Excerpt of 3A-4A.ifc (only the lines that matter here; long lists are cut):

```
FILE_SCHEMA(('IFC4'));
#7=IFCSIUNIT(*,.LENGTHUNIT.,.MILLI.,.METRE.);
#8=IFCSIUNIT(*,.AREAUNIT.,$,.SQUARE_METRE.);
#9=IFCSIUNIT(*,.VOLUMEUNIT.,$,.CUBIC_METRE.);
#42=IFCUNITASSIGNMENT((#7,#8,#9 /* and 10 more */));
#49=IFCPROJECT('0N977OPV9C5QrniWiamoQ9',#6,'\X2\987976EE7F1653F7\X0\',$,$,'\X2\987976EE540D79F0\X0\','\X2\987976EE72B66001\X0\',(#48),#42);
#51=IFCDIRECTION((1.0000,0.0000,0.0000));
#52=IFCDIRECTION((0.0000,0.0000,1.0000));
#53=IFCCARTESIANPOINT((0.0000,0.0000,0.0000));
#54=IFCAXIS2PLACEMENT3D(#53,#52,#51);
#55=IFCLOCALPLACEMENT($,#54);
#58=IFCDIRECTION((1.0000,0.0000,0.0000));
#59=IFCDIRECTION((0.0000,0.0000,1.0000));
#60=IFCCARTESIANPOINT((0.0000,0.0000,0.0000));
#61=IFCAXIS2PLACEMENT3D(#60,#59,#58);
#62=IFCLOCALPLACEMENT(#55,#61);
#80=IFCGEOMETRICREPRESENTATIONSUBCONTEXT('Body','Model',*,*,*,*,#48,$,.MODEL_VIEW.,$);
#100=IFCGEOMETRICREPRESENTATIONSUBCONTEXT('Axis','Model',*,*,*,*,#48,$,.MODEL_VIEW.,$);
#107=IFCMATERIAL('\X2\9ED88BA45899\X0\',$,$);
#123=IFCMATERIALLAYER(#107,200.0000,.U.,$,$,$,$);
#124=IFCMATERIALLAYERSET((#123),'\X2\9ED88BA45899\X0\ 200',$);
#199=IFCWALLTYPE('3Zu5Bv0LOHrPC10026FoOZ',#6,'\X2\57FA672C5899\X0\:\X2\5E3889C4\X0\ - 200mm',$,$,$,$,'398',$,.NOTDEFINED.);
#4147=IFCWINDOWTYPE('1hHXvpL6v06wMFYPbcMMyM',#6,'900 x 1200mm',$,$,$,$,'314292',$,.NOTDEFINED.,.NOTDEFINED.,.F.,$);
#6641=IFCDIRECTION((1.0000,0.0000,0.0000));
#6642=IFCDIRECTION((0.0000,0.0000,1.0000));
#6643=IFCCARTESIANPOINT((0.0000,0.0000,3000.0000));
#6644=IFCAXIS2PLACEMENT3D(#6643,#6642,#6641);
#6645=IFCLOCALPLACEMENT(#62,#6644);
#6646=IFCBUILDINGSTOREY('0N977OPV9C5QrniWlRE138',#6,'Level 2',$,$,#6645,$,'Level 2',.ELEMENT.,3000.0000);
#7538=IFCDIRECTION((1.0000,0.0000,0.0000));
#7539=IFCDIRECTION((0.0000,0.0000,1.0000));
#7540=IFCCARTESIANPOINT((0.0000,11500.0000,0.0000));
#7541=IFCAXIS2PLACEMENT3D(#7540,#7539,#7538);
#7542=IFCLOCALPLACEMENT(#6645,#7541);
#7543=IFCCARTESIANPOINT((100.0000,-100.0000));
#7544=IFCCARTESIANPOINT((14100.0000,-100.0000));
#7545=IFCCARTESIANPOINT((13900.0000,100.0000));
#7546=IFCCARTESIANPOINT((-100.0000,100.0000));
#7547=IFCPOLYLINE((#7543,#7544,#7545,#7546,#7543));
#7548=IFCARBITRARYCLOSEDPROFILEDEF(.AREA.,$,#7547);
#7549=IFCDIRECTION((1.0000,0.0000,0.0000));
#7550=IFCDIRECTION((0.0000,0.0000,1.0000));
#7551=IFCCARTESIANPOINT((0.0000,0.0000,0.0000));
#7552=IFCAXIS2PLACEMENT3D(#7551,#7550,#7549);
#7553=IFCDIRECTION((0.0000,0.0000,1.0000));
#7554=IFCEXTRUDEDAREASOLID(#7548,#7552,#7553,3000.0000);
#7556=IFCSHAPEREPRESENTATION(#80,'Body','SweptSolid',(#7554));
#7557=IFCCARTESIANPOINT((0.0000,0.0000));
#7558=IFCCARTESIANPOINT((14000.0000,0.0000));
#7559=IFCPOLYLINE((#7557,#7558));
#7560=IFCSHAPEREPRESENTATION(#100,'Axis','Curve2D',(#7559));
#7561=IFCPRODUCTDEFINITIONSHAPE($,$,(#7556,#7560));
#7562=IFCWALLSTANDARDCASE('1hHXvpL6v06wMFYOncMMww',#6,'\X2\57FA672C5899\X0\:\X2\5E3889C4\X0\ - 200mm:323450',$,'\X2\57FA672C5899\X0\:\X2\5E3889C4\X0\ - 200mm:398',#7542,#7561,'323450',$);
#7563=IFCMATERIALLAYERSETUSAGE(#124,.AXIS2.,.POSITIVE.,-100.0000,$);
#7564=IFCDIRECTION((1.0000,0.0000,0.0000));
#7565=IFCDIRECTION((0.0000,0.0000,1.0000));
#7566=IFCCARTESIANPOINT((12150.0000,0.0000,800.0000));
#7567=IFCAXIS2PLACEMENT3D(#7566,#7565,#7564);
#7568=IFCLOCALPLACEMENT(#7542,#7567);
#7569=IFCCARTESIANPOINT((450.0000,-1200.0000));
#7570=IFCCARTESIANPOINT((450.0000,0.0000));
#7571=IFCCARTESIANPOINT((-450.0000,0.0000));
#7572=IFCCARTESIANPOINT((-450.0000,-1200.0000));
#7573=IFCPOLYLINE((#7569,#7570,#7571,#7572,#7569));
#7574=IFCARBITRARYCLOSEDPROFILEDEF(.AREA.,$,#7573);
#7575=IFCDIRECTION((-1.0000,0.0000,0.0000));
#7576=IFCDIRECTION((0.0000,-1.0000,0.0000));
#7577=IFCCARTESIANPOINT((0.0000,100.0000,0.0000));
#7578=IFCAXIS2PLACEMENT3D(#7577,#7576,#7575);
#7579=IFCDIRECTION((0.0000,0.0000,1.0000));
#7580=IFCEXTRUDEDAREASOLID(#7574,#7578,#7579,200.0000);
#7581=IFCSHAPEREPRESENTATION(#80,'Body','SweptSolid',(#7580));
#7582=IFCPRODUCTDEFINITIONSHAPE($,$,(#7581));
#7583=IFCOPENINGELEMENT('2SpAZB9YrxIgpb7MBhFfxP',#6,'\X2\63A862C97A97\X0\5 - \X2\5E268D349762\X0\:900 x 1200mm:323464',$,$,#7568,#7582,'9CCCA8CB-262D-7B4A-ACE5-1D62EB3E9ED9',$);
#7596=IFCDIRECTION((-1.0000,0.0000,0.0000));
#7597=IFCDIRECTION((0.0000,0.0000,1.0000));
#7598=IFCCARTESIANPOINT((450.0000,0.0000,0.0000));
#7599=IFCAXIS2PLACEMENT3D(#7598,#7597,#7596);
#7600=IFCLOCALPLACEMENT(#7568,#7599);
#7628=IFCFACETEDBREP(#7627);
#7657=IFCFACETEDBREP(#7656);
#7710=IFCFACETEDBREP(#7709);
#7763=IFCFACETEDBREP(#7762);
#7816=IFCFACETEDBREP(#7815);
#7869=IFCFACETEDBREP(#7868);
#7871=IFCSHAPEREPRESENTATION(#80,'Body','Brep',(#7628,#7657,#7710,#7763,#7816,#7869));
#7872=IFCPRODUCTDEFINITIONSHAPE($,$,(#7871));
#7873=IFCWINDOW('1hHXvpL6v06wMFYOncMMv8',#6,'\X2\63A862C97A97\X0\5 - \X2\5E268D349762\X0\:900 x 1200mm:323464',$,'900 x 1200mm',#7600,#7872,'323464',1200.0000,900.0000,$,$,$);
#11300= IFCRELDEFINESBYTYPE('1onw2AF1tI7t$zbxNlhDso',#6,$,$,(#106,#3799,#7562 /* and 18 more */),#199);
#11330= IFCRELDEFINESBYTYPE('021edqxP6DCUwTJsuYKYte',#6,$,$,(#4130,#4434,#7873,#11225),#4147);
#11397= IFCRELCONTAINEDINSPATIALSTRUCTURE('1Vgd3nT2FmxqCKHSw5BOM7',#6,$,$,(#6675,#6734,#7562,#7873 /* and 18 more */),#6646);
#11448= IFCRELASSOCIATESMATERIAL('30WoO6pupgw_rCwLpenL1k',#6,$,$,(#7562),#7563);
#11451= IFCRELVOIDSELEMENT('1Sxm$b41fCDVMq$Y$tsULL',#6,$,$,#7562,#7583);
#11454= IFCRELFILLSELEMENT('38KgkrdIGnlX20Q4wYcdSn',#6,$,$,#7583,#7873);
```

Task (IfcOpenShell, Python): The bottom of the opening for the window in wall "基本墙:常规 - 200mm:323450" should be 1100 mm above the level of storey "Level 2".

```python
import numpy as np
import ifcopenshell
import ifcopenshell.api.geometry
import ifcopenshell.geom
import ifcopenshell.util.element
import ifcopenshell.util.placement
import ifcopenshell.util.shape
import ifcopenshell.util.unit

model = ifcopenshell.open("3A-4A.ifc")
unit_scale = ifcopenshell.util.unit.calculate_unit_scale(model)

window = model.by_id(7873)
opening = window.FillsVoids[0].RelatingOpeningElement
storey = ifcopenshell.util.element.get_container(window, ifc_class="IfcBuildingStorey")
level = ifcopenshell.util.placement.get_local_placement(storey.ObjectPlacement)[2, 3]

# The opening's origin need not be at the sill, so measure its lowest point.
shape = ifcopenshell.geom.create_shape(ifcopenshell.geom.settings(), opening)
bottom = ifcopenshell.util.shape.get_shape_bottom_elevation(shape, shape.geometry) / unit_scale
dz = level + 1100.0 - bottom

shift = np.array([0.0, 0.0, dz])
# The window is placed relative to its opening, so it follows when the opening moves.
matrix = ifcopenshell.util.placement.get_local_placement(opening.ObjectPlacement)
matrix[:3, 3] += shift
ifcopenshell.api.geometry.edit_object_placement(
    model, product=opening, matrix=matrix, is_si=False, should_transform_children=True
)

print(f"moved by {dz * unit_scale:+.3f} m")

model.write("3A-4A-out.ifc")
```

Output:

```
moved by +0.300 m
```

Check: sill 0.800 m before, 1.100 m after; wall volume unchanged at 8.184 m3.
